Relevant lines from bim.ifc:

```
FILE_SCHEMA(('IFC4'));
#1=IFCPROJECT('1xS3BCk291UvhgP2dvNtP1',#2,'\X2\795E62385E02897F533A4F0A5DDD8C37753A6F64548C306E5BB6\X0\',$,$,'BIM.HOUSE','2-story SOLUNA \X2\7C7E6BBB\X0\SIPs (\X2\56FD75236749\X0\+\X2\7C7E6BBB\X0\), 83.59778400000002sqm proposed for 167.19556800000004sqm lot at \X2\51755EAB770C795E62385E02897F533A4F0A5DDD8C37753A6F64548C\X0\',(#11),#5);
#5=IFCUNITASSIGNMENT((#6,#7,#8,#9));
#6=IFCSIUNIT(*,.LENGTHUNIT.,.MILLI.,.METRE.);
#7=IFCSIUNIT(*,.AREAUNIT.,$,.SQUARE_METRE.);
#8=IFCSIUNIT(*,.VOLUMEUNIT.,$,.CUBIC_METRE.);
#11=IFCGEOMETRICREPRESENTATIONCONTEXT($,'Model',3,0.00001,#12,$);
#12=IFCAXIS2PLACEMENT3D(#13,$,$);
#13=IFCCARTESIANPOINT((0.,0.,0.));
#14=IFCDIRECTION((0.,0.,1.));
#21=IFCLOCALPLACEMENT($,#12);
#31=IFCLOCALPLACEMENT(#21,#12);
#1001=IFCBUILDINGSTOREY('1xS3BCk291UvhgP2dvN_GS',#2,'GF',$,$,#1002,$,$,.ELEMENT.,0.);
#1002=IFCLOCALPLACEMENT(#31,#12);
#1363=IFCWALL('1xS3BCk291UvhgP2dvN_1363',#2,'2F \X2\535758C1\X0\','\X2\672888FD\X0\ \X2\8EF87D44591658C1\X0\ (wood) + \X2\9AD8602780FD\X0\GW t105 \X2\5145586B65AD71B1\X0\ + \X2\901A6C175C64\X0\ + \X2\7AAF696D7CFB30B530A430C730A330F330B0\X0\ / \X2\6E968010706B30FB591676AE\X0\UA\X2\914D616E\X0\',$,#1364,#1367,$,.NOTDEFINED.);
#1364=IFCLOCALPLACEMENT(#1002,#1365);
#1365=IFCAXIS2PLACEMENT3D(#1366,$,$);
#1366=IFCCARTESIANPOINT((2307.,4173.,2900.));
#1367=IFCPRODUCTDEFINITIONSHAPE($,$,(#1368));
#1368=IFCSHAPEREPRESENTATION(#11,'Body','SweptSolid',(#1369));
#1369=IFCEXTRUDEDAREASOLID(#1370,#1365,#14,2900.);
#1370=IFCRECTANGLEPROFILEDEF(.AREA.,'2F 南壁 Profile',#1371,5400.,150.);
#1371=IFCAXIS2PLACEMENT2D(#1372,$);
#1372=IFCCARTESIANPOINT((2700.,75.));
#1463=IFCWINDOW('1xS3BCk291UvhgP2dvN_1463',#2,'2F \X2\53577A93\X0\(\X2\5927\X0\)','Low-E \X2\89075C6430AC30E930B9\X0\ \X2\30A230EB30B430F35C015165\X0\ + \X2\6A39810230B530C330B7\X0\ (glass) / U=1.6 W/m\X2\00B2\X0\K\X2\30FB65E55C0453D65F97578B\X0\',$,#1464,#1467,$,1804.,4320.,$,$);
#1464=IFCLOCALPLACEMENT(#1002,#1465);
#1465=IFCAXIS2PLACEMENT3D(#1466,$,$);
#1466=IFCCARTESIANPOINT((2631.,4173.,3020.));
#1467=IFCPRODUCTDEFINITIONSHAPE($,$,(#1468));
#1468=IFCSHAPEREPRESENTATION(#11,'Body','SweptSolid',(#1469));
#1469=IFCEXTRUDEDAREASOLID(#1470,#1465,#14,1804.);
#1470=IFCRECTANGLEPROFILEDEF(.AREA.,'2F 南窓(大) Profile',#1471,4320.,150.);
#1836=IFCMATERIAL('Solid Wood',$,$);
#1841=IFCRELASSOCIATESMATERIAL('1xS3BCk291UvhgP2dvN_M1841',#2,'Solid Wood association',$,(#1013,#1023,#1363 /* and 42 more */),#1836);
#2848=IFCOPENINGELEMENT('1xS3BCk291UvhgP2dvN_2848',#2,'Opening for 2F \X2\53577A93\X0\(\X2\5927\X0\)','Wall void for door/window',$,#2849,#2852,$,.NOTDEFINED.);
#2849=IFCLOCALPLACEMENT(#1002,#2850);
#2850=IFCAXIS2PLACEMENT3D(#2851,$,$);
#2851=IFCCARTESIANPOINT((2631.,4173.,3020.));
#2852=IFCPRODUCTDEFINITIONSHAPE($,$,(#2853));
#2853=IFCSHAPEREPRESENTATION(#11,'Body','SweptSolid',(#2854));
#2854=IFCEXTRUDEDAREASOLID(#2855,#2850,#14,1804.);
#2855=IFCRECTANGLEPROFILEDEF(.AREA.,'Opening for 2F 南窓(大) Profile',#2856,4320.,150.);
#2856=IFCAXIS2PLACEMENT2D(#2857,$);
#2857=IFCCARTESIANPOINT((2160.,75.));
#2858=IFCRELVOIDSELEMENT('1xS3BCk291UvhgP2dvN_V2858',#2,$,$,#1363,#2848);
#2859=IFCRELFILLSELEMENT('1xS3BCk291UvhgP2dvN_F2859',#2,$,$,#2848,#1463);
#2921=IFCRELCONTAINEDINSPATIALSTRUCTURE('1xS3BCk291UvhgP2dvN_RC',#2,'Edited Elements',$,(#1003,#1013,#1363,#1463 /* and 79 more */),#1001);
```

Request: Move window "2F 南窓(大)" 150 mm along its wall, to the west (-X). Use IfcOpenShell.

```python
import ifcopenshell
import ifcopenshell.api.geometry
import ifcopenshell.util.placement
import ifcopenshell.util.unit

model = ifcopenshell.open("bim.ifc")
unit_scale = ifcopenshell.util.unit.calculate_unit_scale(model)

window = model.by_id(1463)
opening = window.FillsVoids[0].RelatingOpeningElement
wall = opening.VoidsElements[0].RelatingBuildingElement

wall_matrix = ifcopenshell.util.placement.get_local_placement(wall.ObjectPlacement)
shift = wall_matrix[:3, 0] * -0.15 / unit_scale
before = ifcopenshell.util.placement.get_local_placement(window.ObjectPlacement)[:3, 3].copy()

# The window is not placed relative to its opening, so move both.
for product in (opening, window):
    matrix = ifcopenshell.util.placement.get_local_placement(product.ObjectPlacement)
    matrix[:3, 3] += shift
    ifcopenshell.api.geometry.edit_object_placement(model, product=product, matrix=matrix, is_si=False)

after = ifcopenshell.util.placement.get_local_placement(window.ObjectPlacement)[:3, 3]
print("window moved by", (after - before).round(3) + 0.0)

model.write("bim_rev.ifc")
```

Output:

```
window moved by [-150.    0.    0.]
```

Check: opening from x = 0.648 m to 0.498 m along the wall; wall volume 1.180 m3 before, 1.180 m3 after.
